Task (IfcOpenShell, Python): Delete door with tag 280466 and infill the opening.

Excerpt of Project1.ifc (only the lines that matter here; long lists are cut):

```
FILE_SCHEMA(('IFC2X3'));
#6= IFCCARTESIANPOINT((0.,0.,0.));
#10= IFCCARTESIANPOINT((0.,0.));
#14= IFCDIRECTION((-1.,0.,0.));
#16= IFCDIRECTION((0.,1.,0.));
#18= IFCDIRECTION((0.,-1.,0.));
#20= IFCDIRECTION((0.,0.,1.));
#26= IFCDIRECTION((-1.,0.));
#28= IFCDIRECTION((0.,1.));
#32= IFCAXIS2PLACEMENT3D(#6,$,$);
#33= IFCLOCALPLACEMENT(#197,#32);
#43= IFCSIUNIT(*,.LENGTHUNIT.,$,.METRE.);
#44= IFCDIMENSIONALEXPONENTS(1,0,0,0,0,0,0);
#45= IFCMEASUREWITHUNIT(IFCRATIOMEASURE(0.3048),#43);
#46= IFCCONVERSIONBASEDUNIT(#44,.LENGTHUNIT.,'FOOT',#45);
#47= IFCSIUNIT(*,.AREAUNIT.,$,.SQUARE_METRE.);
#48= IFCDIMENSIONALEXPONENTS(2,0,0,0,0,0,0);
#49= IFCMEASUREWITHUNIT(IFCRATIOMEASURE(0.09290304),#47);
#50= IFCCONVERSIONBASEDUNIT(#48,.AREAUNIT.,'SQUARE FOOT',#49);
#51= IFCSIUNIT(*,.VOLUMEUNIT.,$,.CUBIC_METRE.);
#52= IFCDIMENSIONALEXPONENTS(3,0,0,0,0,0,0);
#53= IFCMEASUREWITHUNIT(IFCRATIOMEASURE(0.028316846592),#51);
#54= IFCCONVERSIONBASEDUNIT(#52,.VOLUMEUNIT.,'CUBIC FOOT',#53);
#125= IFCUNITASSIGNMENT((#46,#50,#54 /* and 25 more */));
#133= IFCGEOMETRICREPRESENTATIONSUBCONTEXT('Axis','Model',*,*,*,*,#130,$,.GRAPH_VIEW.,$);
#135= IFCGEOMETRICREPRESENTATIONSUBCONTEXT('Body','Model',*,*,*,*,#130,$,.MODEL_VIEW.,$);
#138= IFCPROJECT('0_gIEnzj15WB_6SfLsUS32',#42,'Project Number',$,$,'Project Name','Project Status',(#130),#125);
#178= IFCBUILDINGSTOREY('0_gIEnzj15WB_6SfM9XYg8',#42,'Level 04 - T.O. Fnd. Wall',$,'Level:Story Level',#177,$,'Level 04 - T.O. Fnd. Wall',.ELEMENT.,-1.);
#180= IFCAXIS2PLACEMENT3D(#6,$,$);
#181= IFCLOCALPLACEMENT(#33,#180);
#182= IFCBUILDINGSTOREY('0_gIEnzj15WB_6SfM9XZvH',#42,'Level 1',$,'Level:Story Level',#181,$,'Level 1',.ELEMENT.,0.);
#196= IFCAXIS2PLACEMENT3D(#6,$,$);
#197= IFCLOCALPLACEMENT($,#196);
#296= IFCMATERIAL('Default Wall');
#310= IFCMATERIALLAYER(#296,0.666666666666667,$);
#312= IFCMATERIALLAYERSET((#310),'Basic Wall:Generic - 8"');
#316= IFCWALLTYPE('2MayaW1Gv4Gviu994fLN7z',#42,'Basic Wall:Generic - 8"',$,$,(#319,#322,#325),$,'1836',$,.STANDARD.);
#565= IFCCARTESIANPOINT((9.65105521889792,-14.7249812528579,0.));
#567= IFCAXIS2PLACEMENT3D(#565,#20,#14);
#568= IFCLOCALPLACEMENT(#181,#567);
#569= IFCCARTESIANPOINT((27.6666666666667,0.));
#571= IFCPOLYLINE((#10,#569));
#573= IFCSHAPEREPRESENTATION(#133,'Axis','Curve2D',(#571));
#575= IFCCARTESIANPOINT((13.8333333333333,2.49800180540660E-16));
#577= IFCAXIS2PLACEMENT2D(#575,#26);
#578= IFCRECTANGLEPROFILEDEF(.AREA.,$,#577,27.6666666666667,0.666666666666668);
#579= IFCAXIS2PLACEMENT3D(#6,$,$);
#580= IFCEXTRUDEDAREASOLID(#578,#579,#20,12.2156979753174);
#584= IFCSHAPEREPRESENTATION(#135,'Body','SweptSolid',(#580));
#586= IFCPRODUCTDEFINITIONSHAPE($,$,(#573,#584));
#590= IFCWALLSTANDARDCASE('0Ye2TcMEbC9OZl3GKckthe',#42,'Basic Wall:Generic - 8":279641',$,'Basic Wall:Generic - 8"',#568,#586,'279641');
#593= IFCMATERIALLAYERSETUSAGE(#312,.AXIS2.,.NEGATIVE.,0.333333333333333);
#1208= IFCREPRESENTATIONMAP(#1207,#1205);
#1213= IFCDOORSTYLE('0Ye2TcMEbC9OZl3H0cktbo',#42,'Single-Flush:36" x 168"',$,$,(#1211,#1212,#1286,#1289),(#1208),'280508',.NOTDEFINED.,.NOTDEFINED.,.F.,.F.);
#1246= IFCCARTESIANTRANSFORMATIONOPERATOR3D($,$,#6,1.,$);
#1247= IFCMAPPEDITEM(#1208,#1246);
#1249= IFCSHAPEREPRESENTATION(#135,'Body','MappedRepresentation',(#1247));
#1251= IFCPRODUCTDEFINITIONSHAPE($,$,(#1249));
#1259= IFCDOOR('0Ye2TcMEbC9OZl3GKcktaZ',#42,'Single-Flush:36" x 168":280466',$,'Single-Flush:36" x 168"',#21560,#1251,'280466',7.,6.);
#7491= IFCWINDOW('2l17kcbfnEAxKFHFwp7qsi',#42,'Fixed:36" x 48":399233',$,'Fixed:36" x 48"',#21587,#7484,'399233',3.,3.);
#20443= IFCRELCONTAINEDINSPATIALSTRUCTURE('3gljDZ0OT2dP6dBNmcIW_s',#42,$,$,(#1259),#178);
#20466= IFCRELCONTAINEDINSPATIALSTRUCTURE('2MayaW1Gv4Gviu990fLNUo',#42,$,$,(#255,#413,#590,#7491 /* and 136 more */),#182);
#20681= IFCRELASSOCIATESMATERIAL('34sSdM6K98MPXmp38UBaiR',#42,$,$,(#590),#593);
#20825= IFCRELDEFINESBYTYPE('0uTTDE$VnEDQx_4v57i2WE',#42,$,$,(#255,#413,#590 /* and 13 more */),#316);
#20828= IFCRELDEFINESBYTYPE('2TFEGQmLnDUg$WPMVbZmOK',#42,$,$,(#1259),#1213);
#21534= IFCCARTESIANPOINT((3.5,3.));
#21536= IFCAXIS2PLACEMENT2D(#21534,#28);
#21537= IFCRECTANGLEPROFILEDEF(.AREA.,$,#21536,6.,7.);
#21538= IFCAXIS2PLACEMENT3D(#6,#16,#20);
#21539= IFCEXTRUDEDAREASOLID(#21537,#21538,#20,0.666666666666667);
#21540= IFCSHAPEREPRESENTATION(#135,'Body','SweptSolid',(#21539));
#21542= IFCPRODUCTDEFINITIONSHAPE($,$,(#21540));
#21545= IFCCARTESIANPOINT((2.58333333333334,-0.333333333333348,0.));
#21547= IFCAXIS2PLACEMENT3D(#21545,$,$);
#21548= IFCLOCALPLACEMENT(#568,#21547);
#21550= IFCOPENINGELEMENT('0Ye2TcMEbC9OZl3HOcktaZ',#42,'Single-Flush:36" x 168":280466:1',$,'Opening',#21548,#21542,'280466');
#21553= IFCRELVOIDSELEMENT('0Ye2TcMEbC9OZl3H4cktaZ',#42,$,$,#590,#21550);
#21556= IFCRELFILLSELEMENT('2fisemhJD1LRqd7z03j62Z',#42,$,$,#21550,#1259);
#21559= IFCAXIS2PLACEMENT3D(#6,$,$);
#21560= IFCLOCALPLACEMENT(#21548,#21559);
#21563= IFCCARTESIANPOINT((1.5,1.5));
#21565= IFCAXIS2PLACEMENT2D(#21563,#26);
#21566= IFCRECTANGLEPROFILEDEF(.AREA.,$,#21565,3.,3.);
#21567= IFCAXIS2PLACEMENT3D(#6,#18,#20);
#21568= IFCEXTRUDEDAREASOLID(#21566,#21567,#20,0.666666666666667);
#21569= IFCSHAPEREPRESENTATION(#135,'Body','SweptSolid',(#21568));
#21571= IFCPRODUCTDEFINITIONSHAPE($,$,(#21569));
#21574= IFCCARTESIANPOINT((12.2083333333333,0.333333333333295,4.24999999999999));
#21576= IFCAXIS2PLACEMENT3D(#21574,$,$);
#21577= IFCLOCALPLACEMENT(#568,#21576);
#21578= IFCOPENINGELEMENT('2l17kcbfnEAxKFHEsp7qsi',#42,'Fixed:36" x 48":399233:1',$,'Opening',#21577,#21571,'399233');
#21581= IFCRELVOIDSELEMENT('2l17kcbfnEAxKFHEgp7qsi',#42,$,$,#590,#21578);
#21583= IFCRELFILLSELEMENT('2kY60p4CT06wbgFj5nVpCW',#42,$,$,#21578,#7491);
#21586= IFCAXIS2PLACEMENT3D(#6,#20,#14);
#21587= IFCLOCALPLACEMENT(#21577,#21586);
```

```python
import ifcopenshell
import ifcopenshell.api.feature
import ifcopenshell.api.root
import ifcopenshell.geom
import ifcopenshell.util.shape

model = ifcopenshell.open("Project1.ifc")
settings = ifcopenshell.geom.settings()


def volume(element):
    """Net volume in cubic metres, openings subtracted."""
    shape = ifcopenshell.geom.create_shape(settings, element)
    return ifcopenshell.util.shape.get_volume(shape.geometry)


door = model.by_guid("0Ye2TcMEbC9OZl3GKcktaZ")
opening = door.FillsVoids[0].RelatingOpeningElement
wall = opening.VoidsElements[0].RelatingBuildingElement
before = volume(wall)

ifcopenshell.api.root.remove_product(model, product=door)
ifcopenshell.api.feature.remove_feature(model, feature=opening)

after = volume(wall)

print(f"wall volume {before:.3f} -> {after:.3f} m3")

model.write("Project1-out.ifc")
```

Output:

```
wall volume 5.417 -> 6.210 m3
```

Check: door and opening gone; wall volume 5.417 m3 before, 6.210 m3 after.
